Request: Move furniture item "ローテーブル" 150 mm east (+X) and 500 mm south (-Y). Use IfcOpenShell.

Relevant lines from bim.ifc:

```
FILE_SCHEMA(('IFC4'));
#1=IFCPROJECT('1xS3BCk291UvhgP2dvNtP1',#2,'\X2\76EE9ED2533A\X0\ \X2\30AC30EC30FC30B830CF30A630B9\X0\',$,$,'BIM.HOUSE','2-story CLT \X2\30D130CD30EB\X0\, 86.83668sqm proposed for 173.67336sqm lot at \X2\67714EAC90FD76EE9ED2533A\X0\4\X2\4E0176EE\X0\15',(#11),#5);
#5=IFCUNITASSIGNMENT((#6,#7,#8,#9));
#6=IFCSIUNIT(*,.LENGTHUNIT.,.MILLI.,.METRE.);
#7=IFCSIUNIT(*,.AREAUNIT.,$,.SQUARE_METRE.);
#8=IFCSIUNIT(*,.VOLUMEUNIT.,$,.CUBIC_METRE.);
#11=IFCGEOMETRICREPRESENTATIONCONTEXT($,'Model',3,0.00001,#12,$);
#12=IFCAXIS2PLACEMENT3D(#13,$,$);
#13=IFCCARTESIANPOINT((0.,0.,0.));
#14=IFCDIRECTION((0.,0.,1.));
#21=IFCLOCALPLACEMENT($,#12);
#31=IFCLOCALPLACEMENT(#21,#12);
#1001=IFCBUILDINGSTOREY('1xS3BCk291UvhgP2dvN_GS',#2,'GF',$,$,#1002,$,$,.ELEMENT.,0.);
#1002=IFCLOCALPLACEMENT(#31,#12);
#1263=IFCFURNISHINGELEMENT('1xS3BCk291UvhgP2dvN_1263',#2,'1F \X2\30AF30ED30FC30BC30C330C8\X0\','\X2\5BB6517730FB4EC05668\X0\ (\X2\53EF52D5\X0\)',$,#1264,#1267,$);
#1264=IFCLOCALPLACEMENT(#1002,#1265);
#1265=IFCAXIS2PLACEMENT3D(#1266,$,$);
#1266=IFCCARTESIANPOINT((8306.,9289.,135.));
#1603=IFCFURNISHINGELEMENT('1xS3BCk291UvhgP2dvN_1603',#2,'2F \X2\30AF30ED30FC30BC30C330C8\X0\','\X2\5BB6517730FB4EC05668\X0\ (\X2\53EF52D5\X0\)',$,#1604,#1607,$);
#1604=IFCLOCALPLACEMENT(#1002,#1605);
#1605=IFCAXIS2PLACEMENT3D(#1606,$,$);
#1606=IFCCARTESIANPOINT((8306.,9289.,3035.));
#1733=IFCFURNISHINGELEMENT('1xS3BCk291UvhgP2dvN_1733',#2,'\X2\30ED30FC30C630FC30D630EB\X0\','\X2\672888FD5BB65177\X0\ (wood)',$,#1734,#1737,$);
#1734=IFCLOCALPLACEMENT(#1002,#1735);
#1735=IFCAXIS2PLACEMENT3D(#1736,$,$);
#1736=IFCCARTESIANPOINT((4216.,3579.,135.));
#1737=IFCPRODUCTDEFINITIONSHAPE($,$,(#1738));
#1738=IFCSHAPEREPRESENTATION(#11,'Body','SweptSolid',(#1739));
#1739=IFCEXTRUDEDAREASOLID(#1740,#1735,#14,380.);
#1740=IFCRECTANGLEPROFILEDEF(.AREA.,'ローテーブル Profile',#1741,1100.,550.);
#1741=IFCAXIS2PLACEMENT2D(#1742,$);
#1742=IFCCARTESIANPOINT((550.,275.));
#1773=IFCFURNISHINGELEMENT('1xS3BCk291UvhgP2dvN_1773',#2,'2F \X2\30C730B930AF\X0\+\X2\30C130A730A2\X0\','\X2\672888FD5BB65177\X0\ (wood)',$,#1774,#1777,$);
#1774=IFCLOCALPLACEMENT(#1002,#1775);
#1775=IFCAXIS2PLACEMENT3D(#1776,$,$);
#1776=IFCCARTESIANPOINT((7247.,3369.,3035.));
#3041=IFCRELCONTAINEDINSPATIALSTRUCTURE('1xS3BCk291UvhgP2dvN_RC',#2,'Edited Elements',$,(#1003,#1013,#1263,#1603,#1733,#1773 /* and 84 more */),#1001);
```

```python
import ifcopenshell
import ifcopenshell.api.geometry
import ifcopenshell.util.placement

model = ifcopenshell.open("bim.ifc")

item = model.by_id(1733)
matrix = ifcopenshell.util.placement.get_local_placement(item.ObjectPlacement)
matrix[0, 3] += 150.0
matrix[1, 3] -= 500.0
ifcopenshell.api.geometry.edit_object_placement(model, product=item, matrix=matrix, is_si=False)

print(ifcopenshell.util.placement.get_local_placement(item.ObjectPlacement).round(3) + 0.0)

model.write("bim_updated.ifc")
```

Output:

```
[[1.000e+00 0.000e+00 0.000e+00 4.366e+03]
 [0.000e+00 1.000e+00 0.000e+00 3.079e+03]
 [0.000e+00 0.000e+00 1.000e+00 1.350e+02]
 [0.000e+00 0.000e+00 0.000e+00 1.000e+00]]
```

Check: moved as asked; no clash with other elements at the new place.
